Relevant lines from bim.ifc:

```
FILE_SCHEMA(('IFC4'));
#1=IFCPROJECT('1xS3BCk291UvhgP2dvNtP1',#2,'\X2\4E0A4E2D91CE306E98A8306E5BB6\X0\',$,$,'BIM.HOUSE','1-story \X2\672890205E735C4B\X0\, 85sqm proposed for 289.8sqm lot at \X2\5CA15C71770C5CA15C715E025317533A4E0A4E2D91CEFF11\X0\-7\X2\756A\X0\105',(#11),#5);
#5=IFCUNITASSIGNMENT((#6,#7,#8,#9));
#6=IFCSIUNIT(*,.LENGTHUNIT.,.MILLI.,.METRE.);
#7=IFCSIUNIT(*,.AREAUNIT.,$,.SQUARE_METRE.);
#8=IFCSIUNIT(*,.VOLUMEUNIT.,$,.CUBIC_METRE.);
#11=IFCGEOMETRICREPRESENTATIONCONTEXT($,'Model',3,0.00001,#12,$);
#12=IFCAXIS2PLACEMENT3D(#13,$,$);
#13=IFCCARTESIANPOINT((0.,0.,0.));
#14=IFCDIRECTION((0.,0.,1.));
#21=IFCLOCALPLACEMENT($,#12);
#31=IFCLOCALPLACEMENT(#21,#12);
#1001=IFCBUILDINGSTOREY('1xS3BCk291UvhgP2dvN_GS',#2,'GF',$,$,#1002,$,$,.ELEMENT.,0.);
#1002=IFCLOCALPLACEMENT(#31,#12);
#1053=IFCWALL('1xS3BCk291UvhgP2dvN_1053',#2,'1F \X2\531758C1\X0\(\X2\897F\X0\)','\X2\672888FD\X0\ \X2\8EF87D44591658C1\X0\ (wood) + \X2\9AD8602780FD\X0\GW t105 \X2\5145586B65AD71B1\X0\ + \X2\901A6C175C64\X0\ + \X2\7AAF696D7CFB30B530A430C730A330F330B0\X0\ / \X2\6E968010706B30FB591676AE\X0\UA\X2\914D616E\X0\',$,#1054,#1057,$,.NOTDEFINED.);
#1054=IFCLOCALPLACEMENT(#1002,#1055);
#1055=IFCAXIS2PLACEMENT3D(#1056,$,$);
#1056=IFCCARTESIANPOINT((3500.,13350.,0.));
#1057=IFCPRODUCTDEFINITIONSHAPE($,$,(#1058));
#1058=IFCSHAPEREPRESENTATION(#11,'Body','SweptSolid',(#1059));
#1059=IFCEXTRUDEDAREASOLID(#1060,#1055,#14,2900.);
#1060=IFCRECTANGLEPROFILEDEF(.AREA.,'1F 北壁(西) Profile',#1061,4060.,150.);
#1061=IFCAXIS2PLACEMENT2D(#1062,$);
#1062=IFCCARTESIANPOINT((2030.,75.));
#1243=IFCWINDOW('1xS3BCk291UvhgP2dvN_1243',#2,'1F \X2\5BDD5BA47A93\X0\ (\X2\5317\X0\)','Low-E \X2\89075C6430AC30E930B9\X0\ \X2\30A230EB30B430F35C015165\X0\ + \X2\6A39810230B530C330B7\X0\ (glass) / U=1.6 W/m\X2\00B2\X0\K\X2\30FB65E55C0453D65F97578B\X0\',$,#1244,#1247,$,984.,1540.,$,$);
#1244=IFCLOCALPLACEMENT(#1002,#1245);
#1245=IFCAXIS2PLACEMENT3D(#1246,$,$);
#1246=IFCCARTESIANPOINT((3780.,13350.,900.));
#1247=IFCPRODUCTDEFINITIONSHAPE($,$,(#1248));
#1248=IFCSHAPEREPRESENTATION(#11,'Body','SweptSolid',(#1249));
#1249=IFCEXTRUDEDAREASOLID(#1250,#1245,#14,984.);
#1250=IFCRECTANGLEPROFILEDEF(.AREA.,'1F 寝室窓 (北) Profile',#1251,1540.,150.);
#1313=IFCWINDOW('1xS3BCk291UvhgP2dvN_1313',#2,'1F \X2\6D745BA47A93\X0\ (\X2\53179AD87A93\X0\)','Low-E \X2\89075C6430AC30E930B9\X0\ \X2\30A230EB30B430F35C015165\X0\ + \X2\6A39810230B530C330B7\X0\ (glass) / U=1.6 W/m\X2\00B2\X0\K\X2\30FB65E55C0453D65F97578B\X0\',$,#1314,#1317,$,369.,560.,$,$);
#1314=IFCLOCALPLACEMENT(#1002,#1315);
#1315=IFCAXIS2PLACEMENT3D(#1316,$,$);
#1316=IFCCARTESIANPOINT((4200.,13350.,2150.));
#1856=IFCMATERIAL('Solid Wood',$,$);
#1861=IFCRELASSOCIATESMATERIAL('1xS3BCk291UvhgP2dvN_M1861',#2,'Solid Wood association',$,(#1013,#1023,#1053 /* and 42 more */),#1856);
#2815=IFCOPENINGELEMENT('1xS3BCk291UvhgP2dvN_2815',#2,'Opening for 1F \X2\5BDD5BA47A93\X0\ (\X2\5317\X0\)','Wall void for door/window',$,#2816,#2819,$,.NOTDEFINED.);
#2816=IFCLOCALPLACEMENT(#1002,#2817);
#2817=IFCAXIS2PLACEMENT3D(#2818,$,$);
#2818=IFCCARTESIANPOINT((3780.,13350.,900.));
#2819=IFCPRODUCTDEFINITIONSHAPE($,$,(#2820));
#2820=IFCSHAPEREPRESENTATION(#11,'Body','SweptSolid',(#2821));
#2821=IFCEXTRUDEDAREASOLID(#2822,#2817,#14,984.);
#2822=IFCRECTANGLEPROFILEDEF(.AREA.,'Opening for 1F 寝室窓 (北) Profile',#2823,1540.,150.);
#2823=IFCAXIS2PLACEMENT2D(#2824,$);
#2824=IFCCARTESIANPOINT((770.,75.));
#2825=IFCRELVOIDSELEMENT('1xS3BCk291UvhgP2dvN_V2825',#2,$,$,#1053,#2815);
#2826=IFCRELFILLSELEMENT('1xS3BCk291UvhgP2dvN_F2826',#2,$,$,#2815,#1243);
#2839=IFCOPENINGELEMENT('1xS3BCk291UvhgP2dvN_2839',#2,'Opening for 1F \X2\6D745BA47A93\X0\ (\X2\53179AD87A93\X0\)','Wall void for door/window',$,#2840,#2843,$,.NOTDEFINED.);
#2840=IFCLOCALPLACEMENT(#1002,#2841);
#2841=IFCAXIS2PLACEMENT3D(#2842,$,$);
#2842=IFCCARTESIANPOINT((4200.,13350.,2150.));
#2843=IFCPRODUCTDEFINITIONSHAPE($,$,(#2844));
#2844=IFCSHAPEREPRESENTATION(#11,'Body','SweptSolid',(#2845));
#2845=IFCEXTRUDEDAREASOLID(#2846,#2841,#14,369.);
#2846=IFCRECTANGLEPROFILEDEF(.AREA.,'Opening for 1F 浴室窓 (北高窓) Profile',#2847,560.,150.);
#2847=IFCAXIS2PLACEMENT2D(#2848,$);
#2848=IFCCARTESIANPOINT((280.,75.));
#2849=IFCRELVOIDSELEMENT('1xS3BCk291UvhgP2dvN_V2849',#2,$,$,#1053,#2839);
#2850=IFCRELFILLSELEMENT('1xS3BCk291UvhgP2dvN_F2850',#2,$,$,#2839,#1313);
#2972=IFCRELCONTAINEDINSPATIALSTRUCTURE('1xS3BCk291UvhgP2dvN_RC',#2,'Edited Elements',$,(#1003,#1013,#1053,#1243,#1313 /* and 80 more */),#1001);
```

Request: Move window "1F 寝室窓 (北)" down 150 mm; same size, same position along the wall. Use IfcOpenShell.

```python
import numpy as np
import ifcopenshell
import ifcopenshell.api.geometry
import ifcopenshell.util.placement
import ifcopenshell.util.unit

model = ifcopenshell.open("bim.ifc")
unit_scale = ifcopenshell.util.unit.calculate_unit_scale(model)

window = model.by_guid("1xS3BCk291UvhgP2dvN_1243")
opening = window.FillsVoids[0].RelatingOpeningElement
dz = -0.15 / unit_scale

shift = np.array([0.0, 0.0, dz])
# The window is not placed relative to its opening, so move both.
for product in (opening, window):
    matrix = ifcopenshell.util.placement.get_local_placement(product.ObjectPlacement)
    matrix[:3, 3] += shift
    ifcopenshell.api.geometry.edit_object_placement(model, product=product, matrix=matrix, is_si=False)

print(f"moved by {dz * unit_scale:+.3f} m")

model.write("bim_v2.ifc")
```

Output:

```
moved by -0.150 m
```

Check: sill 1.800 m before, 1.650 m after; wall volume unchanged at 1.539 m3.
